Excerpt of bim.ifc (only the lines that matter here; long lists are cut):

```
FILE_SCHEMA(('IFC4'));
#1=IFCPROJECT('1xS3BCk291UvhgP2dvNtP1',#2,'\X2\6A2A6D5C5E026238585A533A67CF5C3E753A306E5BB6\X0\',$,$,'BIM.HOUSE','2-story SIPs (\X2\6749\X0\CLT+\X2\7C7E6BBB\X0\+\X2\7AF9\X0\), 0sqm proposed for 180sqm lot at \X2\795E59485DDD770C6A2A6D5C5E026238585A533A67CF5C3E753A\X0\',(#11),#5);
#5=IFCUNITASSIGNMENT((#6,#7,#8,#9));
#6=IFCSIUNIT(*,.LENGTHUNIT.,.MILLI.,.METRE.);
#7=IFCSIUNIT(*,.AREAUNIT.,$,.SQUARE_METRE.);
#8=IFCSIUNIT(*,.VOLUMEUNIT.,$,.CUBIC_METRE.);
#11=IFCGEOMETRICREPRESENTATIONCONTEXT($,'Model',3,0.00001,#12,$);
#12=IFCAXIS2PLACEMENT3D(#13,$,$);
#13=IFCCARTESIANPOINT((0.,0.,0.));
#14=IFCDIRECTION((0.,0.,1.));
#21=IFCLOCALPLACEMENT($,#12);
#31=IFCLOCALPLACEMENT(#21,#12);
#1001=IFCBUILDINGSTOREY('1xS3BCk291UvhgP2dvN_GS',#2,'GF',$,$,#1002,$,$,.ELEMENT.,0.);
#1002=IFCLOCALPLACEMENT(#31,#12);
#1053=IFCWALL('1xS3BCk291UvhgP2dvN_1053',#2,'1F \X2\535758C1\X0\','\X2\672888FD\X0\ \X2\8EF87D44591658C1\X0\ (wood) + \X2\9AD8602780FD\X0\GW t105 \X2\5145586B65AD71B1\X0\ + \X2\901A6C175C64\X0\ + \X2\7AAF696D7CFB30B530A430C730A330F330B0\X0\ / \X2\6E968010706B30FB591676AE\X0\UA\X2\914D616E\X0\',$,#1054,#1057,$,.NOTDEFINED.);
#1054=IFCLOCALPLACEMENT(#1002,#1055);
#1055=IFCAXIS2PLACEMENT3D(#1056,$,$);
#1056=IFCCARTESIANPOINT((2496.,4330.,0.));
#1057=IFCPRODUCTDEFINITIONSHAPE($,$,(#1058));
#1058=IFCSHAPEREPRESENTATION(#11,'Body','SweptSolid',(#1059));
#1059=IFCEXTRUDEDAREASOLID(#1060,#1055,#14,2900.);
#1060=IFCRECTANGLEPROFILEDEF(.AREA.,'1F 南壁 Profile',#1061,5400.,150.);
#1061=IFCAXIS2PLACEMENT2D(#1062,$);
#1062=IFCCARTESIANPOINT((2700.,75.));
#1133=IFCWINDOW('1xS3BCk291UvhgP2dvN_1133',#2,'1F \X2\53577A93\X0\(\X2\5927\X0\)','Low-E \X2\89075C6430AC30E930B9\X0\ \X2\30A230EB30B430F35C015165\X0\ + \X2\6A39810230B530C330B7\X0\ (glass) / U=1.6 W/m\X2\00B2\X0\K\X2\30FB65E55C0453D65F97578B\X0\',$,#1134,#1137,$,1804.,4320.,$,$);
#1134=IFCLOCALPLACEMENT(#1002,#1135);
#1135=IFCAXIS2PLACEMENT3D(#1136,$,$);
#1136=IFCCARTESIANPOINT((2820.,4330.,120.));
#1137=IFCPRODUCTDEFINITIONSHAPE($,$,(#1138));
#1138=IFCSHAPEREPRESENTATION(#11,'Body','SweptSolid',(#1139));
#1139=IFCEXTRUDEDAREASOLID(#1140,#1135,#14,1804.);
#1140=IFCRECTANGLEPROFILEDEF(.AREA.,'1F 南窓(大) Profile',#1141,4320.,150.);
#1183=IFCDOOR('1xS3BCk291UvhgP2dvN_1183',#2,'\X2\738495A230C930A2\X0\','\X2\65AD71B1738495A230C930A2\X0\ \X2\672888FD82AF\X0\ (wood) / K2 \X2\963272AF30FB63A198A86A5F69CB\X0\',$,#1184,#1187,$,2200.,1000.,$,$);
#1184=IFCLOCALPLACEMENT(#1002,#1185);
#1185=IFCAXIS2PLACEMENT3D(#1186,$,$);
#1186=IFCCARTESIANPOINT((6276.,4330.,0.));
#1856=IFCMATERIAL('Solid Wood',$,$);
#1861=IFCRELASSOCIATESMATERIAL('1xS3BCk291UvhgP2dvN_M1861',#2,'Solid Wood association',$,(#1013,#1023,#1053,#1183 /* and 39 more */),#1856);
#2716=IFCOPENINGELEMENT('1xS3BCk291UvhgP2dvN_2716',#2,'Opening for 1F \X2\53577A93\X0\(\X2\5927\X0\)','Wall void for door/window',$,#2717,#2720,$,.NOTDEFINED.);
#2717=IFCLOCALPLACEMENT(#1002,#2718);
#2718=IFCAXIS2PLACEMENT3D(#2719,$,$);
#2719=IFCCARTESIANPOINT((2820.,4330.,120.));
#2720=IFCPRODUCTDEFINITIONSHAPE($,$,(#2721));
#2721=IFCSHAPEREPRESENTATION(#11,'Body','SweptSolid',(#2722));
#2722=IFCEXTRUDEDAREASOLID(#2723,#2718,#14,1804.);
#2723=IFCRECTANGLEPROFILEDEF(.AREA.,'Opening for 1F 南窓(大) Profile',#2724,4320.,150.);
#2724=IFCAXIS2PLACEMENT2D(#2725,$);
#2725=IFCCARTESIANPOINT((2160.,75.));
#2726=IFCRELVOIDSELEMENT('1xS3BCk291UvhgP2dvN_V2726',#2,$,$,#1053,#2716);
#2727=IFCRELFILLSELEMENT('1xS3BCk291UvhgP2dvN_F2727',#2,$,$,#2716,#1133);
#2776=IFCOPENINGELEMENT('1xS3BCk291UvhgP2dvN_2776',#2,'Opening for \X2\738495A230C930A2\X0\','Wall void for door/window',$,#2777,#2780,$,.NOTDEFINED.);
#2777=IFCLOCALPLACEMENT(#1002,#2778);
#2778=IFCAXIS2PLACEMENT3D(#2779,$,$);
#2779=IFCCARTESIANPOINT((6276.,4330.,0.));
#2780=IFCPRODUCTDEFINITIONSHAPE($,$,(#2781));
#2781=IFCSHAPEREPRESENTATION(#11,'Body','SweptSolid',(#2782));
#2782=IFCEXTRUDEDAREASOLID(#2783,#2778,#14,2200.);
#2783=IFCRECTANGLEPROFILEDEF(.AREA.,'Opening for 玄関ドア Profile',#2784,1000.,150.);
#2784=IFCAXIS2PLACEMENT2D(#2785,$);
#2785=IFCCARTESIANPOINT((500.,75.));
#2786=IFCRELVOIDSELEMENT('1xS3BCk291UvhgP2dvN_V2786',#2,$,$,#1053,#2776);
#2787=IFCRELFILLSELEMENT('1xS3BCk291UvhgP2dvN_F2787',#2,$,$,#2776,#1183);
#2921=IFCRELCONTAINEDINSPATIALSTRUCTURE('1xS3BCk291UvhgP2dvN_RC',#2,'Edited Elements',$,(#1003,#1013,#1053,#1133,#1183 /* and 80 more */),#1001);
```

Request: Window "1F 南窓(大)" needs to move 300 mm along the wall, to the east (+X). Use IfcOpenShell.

```python
import ifcopenshell
import ifcopenshell.api.geometry
import ifcopenshell.util.placement

model = ifcopenshell.open("bim.ifc")

window = model.by_guid("1xS3BCk291UvhgP2dvN_1133")
opening = window.FillsVoids[0].RelatingOpeningElement
wall = opening.VoidsElements[0].RelatingBuildingElement

wall_matrix = ifcopenshell.util.placement.get_local_placement(wall.ObjectPlacement)
shift = wall_matrix[:3, 0] * 300.0
before = ifcopenshell.util.placement.get_local_placement(window.ObjectPlacement)[:3, 3].copy()

# The window is not placed relative to its opening, so move both.
for product in (opening, window):
    matrix = ifcopenshell.util.placement.get_local_placement(product.ObjectPlacement)
    matrix[:3, 3] += shift
    ifcopenshell.api.geometry.edit_object_placement(model, product=product, matrix=matrix, is_si=False)

after = ifcopenshell.util.placement.get_local_placement(window.ObjectPlacement)[:3, 3]
print("window moved by", (after - before).round(3) + 0.0)

model.write("bim_rev.ifc")
```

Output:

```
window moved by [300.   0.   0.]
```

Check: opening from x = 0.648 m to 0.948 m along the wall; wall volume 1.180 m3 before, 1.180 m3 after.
